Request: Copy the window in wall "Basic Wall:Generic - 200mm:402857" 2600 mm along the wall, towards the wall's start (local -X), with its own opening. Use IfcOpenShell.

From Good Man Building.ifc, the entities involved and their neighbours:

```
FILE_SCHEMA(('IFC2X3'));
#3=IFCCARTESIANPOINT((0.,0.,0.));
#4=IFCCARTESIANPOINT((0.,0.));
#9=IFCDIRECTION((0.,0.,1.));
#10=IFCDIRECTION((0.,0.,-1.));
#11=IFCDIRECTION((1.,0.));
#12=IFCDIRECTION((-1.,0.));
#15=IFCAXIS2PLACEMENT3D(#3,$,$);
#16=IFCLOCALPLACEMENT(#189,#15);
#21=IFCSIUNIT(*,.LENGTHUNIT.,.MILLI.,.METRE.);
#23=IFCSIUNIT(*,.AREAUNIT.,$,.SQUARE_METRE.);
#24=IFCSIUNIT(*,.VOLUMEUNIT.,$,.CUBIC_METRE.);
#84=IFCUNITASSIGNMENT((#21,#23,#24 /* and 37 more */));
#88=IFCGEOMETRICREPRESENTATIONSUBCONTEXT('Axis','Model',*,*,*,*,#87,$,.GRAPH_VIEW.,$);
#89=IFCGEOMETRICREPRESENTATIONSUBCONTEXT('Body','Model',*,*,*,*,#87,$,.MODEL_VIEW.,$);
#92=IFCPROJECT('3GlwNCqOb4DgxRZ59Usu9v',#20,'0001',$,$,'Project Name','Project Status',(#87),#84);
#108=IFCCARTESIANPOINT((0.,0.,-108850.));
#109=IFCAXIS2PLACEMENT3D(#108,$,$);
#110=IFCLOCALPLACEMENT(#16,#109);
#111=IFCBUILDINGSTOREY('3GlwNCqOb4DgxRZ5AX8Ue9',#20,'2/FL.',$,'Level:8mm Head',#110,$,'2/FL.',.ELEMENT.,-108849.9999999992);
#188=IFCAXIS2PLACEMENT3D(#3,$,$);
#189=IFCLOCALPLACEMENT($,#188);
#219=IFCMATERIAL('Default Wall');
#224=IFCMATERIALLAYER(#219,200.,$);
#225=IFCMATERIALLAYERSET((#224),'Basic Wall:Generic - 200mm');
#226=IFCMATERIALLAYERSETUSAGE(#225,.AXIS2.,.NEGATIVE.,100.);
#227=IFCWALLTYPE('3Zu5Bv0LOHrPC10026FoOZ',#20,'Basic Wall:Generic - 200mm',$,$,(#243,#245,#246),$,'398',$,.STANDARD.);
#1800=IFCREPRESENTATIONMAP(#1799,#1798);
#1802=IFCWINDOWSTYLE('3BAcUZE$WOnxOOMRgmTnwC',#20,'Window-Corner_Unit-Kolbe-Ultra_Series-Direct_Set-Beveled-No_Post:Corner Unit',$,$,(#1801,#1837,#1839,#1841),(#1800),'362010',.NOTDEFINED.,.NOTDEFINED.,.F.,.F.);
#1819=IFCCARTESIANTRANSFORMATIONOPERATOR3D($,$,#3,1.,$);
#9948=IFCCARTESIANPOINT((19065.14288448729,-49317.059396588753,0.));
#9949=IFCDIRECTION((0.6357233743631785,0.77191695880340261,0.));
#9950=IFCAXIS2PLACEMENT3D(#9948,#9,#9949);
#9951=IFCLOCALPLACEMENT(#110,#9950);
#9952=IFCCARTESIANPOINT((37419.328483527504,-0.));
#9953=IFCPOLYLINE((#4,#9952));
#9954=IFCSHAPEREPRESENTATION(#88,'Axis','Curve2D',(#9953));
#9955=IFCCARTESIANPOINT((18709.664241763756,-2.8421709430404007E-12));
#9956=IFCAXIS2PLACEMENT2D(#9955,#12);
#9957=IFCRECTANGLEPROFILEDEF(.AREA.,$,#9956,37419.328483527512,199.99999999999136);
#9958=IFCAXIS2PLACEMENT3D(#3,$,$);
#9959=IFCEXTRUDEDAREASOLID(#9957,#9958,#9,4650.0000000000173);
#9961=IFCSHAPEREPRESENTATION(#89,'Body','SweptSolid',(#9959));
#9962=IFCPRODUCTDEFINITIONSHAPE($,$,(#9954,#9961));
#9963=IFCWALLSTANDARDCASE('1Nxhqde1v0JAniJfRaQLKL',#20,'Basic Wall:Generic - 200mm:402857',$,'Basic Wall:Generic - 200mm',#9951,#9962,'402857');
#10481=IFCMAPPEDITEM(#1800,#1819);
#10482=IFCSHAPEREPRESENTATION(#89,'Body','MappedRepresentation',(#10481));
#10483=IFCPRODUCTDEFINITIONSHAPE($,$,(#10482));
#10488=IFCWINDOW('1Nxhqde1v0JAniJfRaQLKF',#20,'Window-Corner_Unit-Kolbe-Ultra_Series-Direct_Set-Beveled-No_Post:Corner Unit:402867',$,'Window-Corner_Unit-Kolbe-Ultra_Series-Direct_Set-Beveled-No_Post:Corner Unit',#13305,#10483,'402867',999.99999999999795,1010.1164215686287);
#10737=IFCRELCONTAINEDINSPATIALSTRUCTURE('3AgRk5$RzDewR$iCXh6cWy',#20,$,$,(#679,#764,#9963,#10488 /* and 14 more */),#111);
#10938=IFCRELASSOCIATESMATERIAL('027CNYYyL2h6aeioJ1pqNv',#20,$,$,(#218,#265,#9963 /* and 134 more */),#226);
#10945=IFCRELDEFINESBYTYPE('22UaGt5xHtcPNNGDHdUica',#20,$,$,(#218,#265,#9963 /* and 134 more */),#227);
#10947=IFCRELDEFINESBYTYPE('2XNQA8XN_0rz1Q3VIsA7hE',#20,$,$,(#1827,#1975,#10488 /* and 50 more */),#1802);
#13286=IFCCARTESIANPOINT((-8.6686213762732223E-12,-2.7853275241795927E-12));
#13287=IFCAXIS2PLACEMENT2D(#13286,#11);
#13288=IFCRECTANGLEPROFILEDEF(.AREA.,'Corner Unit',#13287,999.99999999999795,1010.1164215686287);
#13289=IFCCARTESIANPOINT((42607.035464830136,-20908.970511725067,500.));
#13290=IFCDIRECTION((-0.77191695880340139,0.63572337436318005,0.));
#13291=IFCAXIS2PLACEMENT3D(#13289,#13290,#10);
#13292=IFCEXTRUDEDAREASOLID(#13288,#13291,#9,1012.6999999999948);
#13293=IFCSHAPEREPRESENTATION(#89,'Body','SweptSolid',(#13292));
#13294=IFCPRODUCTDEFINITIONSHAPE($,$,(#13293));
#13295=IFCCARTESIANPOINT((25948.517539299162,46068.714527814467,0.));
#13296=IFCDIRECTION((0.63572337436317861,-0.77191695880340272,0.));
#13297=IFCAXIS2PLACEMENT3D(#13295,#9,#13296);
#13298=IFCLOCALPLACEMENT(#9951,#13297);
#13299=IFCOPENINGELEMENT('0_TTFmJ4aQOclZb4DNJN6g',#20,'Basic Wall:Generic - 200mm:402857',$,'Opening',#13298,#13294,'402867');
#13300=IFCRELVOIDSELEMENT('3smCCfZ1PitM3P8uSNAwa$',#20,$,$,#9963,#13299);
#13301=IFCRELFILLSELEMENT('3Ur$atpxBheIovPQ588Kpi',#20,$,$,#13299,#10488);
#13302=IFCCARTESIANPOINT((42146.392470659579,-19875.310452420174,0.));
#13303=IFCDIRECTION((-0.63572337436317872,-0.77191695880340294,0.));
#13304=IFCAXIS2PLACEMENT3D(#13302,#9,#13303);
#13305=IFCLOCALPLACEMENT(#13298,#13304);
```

```python
import ifcopenshell
import ifcopenshell.api.feature
import ifcopenshell.api.geometry
import ifcopenshell.api.root
import ifcopenshell.geom
import ifcopenshell.util.element
import ifcopenshell.util.placement
import ifcopenshell.util.shape

model = ifcopenshell.open("Good Man Building.ifc")
settings = ifcopenshell.geom.settings()


def volume(element):
    """Net volume in cubic metres, openings subtracted."""
    shape = ifcopenshell.geom.create_shape(settings, element)
    return ifcopenshell.util.shape.get_volume(shape.geometry)


def reuse_history(source, copy):
    """copy_class also copies each property set's owner history, people and application; keep the originals."""
    for rel in copy.IsDefinedBy:
        if rel.is_a("IfcRelDefinesByProperties") and (history := rel.RelatingPropertyDefinition.OwnerHistory):
            rel.RelatingPropertyDefinition.OwnerHistory = source.OwnerHistory
            ifcopenshell.util.element.remove_deep2(model, history)


window = model.by_guid("1Nxhqde1v0JAniJfRaQLKF")
opening = window.FillsVoids[0].RelatingOpeningElement
wall = opening.VoidsElements[0].RelatingBuildingElement
before = volume(wall)
shift = ifcopenshell.util.placement.get_local_placement(wall.ObjectPlacement)[:3, 0] * -2600.0

# copy_class copies the void relationship, type, container and properties, but no geometry.
new_opening = ifcopenshell.api.root.copy_class(model, product=opening)
new_opening.Representation = ifcopenshell.util.element.copy_deep(
    model, opening.Representation, exclude=["IfcGeometricRepresentationContext", "IfcRepresentationMap"]
)
new_opening.Name = "Basic Wall:Generic - 200mm"
new_opening.Tag = None
new_window = ifcopenshell.api.root.copy_class(model, product=window)
new_window.Representation = ifcopenshell.util.element.copy_deep(
    model, window.Representation, exclude=["IfcGeometricRepresentationContext", "IfcRepresentationMap"]
)
new_window.Name = "Window-Corner_Unit-Kolbe-Ultra_Series-Direct_Set-Beveled-No_Post:Corner Unit"
new_window.Tag = None
reuse_history(window, new_window)
fills = ifcopenshell.api.feature.add_filling(model, opening=new_opening, element=new_window)
fills.OwnerHistory = new_window.OwnerHistory  # required in IFC2X3

for old, new in ((opening, new_opening), (window, new_window)):
    matrix = ifcopenshell.util.placement.get_local_placement(old.ObjectPlacement)
    matrix[:3, 3] += shift
    ifcopenshell.api.geometry.edit_object_placement(model, product=new, matrix=matrix, is_si=False)

after = volume(wall)

print(f"wall volume {before:.3f} -> {after:.3f} m3")

model.write("Good Man Building_rev.ifc")
```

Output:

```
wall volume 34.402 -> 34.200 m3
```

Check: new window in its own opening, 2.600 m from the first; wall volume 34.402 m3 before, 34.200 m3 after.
